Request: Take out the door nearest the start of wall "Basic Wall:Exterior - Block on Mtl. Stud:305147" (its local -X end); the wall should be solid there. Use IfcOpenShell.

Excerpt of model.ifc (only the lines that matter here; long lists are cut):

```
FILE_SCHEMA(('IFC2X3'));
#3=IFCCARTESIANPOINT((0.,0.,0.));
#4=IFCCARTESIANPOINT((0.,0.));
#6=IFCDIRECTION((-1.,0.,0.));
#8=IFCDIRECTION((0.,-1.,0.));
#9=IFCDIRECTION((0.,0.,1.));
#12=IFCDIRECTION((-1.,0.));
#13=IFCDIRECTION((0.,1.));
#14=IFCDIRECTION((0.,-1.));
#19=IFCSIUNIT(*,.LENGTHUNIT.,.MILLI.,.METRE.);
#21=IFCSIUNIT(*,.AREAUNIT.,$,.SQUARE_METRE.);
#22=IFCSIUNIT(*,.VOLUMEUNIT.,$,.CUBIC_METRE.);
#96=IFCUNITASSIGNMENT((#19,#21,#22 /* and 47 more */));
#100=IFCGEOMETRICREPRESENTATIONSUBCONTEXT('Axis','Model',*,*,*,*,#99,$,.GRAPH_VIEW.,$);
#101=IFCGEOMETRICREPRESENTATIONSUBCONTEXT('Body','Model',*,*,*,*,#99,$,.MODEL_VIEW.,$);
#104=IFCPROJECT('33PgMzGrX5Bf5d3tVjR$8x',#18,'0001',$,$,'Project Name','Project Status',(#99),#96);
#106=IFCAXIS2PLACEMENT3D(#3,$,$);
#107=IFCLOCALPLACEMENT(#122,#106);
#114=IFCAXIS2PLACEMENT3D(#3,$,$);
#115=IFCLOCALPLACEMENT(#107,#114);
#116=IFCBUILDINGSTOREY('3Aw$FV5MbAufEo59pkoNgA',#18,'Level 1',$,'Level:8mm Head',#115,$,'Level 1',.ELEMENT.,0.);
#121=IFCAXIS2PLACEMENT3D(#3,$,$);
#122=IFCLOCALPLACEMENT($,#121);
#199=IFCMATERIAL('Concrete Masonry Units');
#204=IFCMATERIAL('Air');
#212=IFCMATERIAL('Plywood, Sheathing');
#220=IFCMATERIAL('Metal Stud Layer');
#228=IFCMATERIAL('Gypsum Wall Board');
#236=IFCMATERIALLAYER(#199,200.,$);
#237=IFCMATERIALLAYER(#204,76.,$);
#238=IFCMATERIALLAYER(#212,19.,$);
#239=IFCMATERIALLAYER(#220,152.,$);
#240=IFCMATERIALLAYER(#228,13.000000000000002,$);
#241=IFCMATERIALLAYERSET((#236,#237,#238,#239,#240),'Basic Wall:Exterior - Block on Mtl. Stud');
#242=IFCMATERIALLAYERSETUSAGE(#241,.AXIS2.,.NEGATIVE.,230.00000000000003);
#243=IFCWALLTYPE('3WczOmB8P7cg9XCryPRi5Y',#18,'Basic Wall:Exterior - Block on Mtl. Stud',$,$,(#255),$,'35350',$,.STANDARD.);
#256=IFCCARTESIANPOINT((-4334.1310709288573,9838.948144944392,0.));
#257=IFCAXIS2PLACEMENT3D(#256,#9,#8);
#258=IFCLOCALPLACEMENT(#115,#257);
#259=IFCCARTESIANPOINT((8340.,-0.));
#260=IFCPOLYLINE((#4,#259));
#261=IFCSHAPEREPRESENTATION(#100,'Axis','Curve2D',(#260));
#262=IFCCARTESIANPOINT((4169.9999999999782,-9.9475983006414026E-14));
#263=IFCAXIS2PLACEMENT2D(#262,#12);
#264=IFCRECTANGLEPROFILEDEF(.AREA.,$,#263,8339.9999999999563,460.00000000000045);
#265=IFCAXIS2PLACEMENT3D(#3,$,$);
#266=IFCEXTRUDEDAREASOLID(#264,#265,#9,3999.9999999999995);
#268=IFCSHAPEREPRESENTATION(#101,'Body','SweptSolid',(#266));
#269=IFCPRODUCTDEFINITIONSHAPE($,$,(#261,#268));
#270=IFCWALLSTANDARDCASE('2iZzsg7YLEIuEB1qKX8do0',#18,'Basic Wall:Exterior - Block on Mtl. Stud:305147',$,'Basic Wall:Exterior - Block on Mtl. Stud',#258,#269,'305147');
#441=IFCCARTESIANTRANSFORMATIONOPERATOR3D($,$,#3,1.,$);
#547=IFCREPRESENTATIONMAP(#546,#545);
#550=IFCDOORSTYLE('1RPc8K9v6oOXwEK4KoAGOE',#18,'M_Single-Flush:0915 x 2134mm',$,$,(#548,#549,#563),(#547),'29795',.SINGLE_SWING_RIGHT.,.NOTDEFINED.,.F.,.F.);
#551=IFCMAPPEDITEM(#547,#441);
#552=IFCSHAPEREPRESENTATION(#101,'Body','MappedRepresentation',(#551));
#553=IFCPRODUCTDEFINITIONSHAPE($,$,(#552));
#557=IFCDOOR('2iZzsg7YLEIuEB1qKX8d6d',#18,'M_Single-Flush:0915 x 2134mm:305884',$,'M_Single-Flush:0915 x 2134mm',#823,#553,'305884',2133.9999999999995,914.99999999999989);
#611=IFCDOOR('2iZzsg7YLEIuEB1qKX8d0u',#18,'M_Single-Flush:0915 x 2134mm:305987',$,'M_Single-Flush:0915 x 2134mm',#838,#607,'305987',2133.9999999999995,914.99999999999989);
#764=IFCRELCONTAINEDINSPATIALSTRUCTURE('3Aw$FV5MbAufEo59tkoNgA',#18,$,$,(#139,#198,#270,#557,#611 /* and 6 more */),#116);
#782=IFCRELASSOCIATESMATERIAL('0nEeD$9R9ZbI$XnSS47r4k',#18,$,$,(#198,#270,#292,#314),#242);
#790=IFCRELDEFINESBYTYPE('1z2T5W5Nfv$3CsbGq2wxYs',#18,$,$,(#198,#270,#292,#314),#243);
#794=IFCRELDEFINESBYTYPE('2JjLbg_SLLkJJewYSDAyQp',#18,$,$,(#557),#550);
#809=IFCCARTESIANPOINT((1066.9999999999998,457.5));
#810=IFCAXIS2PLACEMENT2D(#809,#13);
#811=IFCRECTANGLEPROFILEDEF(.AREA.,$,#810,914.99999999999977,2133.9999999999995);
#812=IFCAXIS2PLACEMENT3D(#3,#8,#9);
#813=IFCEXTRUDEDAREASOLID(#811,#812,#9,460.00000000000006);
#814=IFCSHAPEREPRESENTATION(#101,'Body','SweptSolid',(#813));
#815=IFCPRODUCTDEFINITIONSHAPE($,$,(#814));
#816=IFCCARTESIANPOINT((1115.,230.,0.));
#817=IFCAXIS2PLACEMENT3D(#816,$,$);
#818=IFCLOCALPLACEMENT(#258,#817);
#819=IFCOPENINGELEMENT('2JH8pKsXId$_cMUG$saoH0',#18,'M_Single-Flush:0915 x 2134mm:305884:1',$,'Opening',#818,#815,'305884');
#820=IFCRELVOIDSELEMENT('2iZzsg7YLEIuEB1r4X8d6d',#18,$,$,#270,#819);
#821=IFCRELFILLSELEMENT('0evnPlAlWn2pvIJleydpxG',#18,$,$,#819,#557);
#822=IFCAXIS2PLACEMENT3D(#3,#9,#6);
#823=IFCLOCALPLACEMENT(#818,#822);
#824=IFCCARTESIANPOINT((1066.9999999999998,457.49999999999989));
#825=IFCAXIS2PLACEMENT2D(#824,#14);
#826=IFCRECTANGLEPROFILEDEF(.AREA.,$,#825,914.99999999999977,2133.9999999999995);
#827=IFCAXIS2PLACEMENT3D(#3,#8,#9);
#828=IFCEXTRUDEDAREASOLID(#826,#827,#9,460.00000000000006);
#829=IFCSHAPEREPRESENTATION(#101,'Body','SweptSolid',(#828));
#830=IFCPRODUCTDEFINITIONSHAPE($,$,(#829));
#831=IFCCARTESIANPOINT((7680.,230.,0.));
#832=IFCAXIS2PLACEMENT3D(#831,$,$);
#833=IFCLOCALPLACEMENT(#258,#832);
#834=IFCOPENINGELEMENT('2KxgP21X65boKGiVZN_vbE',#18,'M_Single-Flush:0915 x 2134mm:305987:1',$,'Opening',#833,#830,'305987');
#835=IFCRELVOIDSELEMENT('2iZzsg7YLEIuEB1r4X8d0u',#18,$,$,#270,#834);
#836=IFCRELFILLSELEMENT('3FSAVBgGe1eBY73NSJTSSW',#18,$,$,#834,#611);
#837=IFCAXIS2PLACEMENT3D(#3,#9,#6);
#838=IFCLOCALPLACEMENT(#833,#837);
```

```python
import ifcopenshell
import ifcopenshell.api.feature
import ifcopenshell.api.root
import ifcopenshell.geom
import ifcopenshell.util.shape

model = ifcopenshell.open("model.ifc")
settings = ifcopenshell.geom.settings()


def volume(element):
    """Net volume in cubic metres, openings subtracted."""
    shape = ifcopenshell.geom.create_shape(settings, element)
    return ifcopenshell.util.shape.get_volume(shape.geometry)


door = model.by_guid("2iZzsg7YLEIuEB1qKX8d6d")
opening = door.FillsVoids[0].RelatingOpeningElement
wall = opening.VoidsElements[0].RelatingBuildingElement
before = volume(wall)

ifcopenshell.api.root.remove_product(model, product=door)
ifcopenshell.api.feature.remove_feature(model, feature=opening)

after = volume(wall)

print(f"wall volume {before:.3f} -> {after:.3f} m3")

model.write("model-out.ifc")
```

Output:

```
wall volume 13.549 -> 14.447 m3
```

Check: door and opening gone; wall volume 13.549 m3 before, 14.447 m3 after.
